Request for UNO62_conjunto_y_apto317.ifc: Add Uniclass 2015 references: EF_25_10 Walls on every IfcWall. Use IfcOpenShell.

First a look at what the model holds.

```python
import ifcopenshell

model = ifcopenshell.open("UNO62_conjunto_y_apto317.ifc")
print(model.schema)
print("classifications:", [c.Name for c in model.by_type("IfcClassification")])
for ifc_class in ("IfcDoor", "IfcRoof", "IfcStair", "IfcWall", "IfcWindow"):
    print(ifc_class, len(model.by_type(ifc_class)))
```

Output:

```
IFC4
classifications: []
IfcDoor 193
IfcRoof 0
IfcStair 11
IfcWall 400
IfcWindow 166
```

```python
import ifcopenshell
import ifcopenshell.api.classification

model = ifcopenshell.open("UNO62_conjunto_y_apto317.ifc")

system = ifcopenshell.api.classification.add_classification(model, classification="Uniclass 2015")

codes = {
    "IfcWall": ("EF_25_10", "Walls"),
}
for ifc_class, (code, name) in codes.items():
    products = model.by_type(ifc_class)
    ifcopenshell.api.classification.add_reference(
        model, products=products, classification=system, identification=code, name=name
    )
    print(code, len(products))

model.write("UNO62_conjunto_y_apto317_v2.ifc")
```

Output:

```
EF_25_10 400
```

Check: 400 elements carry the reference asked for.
